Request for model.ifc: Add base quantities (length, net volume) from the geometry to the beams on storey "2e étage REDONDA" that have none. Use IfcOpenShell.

First a look at what the model holds.

```python
import ifcopenshell
import ifcopenshell.util.element
import ifcopenshell.util.unit

model = ifcopenshell.open("model.ifc")
print(model.schema)
for unit_type in ("LENGTHUNIT", "AREAUNIT", "VOLUMEUNIT"):
    print(unit_type, ifcopenshell.util.unit.calculate_unit_scale(model, unit_type))
storey = next(s for s in model.by_type("IfcBuildingStorey") if s.Name == "2e étage REDONDA")
beams = [e for e in ifcopenshell.util.element.get_decomposition(storey) if e.is_a("IfcBeam")]
for e in sorted(beams, key=lambda e: e.id()):
    print(e.id(), e.is_a(), e.Name, list(ifcopenshell.util.element.get_psets(e, qtos_only=True)), sep=" | ")
```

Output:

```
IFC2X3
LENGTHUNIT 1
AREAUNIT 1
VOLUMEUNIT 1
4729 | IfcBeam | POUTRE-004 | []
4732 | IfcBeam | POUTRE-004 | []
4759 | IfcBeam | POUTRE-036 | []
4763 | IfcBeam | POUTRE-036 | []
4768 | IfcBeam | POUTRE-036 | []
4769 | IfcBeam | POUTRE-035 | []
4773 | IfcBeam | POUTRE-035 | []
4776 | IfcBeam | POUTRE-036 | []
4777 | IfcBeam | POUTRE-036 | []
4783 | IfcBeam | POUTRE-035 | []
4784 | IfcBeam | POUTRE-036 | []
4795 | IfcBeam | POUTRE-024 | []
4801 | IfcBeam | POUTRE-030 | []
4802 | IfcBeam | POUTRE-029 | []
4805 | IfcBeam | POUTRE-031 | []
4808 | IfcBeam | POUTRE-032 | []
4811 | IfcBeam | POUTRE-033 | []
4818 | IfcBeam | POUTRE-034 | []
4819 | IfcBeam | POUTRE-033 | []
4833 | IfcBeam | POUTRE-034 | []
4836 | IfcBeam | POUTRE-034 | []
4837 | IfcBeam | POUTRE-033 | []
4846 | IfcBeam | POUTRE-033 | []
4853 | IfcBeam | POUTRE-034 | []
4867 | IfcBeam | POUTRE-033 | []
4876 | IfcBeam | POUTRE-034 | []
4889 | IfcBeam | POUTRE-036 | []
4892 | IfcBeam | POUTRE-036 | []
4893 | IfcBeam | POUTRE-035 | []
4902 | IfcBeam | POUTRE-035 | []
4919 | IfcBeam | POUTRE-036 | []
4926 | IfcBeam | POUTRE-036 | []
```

```python
import ifcopenshell
import ifcopenshell.api.pset
import ifcopenshell.geom
import ifcopenshell.util.element
import ifcopenshell.util.shape
import ifcopenshell.util.unit

model = ifcopenshell.open("model.ifc")
unit_scale = ifcopenshell.util.unit.calculate_unit_scale(model)
volume_scale = ifcopenshell.util.unit.calculate_unit_scale(model, "VOLUMEUNIT")
settings = ifcopenshell.geom.settings()

storey = next(s for s in model.by_type("IfcBuildingStorey") if s.Name == "2e étage REDONDA")
beams = [e for e in ifcopenshell.util.element.get_decomposition(storey) if e.is_a("IfcBeam")]

for e in sorted(beams, key=lambda e: e.id()):
    if ifcopenshell.util.element.get_psets(e, qtos_only=True, should_inherit=False):
        continue
    # Geometry comes back in metres, in the element's own axes.
    shape = ifcopenshell.geom.create_shape(settings, e)
    values = {
        "Length": ifcopenshell.util.shape.get_max_xyz(shape.geometry) / unit_scale,
        "NetVolume": ifcopenshell.util.shape.get_volume(shape.geometry) / volume_scale,
    }
    qto = ifcopenshell.api.pset.add_qto(model, product=e, name="BaseQuantities")
    ifcopenshell.api.pset.edit_qto(model, qto=qto, properties=values)
    print(e.id(), {k: round(v, 3) for k, v in values.items()})

model.write("model_rev.ifc")
```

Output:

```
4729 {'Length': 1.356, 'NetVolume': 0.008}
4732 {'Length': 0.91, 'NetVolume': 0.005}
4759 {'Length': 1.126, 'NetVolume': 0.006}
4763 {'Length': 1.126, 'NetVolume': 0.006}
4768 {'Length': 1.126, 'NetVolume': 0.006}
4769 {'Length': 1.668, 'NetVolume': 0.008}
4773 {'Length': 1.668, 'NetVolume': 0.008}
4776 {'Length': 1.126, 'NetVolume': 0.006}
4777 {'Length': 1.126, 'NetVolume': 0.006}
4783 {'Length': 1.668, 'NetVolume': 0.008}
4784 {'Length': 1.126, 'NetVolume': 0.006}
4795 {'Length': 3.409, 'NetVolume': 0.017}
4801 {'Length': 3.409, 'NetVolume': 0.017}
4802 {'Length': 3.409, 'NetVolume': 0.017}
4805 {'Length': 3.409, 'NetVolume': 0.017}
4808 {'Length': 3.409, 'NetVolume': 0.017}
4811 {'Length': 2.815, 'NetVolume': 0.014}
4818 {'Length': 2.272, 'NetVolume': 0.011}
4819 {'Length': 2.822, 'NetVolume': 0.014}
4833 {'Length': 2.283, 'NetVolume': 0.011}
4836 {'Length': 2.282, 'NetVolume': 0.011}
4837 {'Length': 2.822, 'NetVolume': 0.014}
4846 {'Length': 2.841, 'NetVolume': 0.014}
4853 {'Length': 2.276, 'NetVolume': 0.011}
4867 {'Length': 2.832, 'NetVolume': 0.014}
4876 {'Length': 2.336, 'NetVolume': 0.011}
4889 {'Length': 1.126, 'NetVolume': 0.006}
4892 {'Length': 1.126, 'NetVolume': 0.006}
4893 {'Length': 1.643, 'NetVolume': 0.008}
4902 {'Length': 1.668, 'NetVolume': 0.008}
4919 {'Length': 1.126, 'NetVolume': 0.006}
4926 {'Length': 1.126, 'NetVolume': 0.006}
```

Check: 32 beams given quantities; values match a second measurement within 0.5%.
